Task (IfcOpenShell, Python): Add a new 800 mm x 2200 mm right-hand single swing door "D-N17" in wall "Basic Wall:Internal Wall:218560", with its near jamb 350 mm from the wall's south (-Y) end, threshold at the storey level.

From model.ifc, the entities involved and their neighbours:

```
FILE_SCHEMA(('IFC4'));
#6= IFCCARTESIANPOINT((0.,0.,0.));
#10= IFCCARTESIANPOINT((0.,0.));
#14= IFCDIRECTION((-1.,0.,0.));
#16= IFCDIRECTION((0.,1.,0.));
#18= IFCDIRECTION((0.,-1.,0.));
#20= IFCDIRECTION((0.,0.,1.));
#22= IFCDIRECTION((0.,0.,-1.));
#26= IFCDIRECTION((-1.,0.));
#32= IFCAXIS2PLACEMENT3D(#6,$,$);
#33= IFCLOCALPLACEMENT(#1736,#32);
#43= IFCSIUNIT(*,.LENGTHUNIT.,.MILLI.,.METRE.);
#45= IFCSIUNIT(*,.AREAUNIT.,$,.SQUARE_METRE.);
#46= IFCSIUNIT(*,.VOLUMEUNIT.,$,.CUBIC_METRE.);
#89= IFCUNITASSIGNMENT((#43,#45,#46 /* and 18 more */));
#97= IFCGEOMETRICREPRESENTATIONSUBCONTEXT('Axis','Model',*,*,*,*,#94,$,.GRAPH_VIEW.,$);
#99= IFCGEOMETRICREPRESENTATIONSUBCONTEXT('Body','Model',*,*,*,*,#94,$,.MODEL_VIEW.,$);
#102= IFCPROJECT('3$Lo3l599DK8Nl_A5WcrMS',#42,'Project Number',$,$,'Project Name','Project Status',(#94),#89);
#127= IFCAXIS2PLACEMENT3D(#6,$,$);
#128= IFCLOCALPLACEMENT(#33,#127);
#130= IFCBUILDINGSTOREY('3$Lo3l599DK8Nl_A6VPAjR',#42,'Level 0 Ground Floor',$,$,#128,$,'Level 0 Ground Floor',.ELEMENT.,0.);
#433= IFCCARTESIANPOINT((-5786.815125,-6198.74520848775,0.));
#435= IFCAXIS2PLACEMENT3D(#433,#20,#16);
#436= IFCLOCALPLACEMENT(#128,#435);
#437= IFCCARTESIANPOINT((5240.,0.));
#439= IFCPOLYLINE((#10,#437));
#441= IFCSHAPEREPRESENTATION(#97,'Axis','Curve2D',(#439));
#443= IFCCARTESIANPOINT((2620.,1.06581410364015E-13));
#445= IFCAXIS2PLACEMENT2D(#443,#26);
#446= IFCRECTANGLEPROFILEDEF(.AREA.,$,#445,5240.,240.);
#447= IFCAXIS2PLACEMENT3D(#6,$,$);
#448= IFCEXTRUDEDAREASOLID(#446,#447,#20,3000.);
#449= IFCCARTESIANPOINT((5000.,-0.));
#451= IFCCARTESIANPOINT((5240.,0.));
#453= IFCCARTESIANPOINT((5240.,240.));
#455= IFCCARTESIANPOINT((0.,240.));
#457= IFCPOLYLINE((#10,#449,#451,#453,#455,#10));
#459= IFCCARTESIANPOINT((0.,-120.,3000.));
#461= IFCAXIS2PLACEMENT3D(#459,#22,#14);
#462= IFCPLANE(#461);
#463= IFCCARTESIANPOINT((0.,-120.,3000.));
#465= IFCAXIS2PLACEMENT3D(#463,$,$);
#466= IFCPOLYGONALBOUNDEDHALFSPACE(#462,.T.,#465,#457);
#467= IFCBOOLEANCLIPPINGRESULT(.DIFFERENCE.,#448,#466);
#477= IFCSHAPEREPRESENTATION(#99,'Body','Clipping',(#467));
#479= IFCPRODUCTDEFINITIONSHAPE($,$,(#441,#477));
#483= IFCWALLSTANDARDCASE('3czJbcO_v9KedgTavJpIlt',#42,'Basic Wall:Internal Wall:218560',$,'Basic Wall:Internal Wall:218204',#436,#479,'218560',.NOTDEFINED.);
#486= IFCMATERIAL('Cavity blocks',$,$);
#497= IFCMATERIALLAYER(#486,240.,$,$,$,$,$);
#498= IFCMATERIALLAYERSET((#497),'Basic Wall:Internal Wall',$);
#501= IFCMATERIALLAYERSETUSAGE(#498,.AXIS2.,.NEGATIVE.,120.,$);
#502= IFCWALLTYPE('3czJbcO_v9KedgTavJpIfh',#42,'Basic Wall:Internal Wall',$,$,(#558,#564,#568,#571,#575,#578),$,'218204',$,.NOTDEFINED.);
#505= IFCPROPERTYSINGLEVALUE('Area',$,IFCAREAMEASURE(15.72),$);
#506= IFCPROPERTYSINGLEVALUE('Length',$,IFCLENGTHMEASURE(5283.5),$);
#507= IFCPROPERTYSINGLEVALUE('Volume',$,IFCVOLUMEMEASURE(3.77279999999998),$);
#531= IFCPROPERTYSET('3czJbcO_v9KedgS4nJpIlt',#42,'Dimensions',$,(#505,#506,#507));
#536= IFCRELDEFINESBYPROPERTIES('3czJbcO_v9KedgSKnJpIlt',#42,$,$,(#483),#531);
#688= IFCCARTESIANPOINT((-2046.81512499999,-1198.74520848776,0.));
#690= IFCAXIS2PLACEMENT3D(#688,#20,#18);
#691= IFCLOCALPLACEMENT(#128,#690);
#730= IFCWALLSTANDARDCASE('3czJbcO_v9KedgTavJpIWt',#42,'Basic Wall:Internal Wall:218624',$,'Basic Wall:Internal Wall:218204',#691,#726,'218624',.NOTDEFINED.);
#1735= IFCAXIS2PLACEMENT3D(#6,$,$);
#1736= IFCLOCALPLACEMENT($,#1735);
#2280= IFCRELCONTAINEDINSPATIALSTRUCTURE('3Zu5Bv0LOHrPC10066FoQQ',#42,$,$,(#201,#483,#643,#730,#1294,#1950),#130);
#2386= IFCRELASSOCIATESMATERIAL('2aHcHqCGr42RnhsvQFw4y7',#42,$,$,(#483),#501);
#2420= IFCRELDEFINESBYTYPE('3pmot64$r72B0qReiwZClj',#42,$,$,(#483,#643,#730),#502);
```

```python
import numpy as np
import ifcopenshell
import ifcopenshell.api.feature
import ifcopenshell.api.geometry
import ifcopenshell.api.pset
import ifcopenshell.api.root
import ifcopenshell.api.spatial
import ifcopenshell.geom
import ifcopenshell.util.element
import ifcopenshell.util.placement
import ifcopenshell.util.representation
import ifcopenshell.util.shape
import ifcopenshell.util.unit

model = ifcopenshell.open("model.ifc")
unit_scale = ifcopenshell.util.unit.calculate_unit_scale(model)
area_scale = ifcopenshell.util.unit.calculate_unit_scale(model, "AREAUNIT")
volume_scale = ifcopenshell.util.unit.calculate_unit_scale(model, "VOLUMEUNIT")
settings = ifcopenshell.geom.settings()


def volume(element):
    """Net volume in cubic metres, openings subtracted."""
    shape = ifcopenshell.geom.create_shape(settings, element)
    return ifcopenshell.util.shape.get_volume(shape.geometry)


wall = model.by_guid("3czJbcO_v9KedgTavJpIlt")
storey = ifcopenshell.util.element.get_container(wall, ifc_class="IfcBuildingStorey")
context = ifcopenshell.util.representation.get_context(model, "Model", "Body", "MODEL_VIEW")
before = volume(wall)

width, height, from_end, sill = 0.8, 2.2, 0.35, 0.0  # metres

# The wall runs along its own X axis, and the end named is its -X end.
wall_shape = ifcopenshell.geom.create_shape(settings, wall)
x, y, z = ifcopenshell.util.shape.get_vertices(wall_shape.geometry).T
start = x.min() + from_end
face, thickness = float(y.min()), float(y.max() - y.min())
wall_matrix = ifcopenshell.util.placement.get_local_placement(wall.ObjectPlacement)
level = ifcopenshell.util.placement.get_local_placement(storey.ObjectPlacement)[2, 3]


def in_wall(x, y):
    """Placement at x, y metres in the wall's axes, at sill height."""
    matrix = wall_matrix.copy()
    matrix[:, 3] = wall_matrix @ np.array([x / unit_scale, y / unit_scale, 0.0, 1.0])
    matrix[2, 3] = level + sill / unit_scale
    return matrix


# Opening: a box that overshoots both wall faces by 50 mm.
opening = ifcopenshell.api.root.create_entity(model, ifc_class="IfcOpeningElement", predefined_type="OPENING")
box = ifcopenshell.api.geometry.add_wall_representation(
    model, context=context, length=width, height=height, thickness=thickness + 0.1
)
ifcopenshell.api.geometry.assign_representation(model, product=opening, representation=box)
ifcopenshell.api.geometry.edit_object_placement(model, product=opening, matrix=in_wall(start, face - 0.05), is_si=False)
ifcopenshell.api.feature.add_feature(model, feature=opening, element=wall)

door = ifcopenshell.api.root.create_entity(model, ifc_class="IfcDoor", name="D-N17", predefined_type="DOOR")
door.OverallWidth, door.OverallHeight = width / unit_scale, height / unit_scale
door.OperationType = "SINGLE_SWING_RIGHT"
body = ifcopenshell.api.geometry.add_door_representation(
    model,
    context=context,
    overall_width=door.OverallWidth,
    overall_height=door.OverallHeight,
    operation_type="SINGLE_SWING_RIGHT",
    lining_properties={"LiningDepth": thickness / unit_scale, "ThresholdDepth": thickness / unit_scale},
)
ifcopenshell.api.geometry.assign_representation(model, product=door, representation=body)
ifcopenshell.api.spatial.assign_container(model, products=[door], relating_structure=storey)
ifcopenshell.api.feature.add_filling(model, opening=opening, element=door)

# The lining spans the wall, so the door starts at the wall face.
ifcopenshell.api.geometry.edit_object_placement(model, product=door, matrix=in_wall(start, face), is_si=False)

after = volume(wall)

# Update the wall's stored quantities.
pset = model.by_id(ifcopenshell.util.element.get_pset(wall, "Dimensions", should_inherit=False)["id"])
ifcopenshell.api.pset.edit_pset(model, pset=pset, properties={
    "Area": model.create_entity("IfcAreaMeasure", after / thickness / area_scale),
    "Volume": model.create_entity("IfcVolumeMeasure", after / volume_scale),
})

print(f"wall volume {before:.3f} -> {after:.3f} m3")

model.write("model_edited.ifc")
```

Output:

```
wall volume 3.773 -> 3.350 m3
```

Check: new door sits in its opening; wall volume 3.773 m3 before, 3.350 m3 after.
